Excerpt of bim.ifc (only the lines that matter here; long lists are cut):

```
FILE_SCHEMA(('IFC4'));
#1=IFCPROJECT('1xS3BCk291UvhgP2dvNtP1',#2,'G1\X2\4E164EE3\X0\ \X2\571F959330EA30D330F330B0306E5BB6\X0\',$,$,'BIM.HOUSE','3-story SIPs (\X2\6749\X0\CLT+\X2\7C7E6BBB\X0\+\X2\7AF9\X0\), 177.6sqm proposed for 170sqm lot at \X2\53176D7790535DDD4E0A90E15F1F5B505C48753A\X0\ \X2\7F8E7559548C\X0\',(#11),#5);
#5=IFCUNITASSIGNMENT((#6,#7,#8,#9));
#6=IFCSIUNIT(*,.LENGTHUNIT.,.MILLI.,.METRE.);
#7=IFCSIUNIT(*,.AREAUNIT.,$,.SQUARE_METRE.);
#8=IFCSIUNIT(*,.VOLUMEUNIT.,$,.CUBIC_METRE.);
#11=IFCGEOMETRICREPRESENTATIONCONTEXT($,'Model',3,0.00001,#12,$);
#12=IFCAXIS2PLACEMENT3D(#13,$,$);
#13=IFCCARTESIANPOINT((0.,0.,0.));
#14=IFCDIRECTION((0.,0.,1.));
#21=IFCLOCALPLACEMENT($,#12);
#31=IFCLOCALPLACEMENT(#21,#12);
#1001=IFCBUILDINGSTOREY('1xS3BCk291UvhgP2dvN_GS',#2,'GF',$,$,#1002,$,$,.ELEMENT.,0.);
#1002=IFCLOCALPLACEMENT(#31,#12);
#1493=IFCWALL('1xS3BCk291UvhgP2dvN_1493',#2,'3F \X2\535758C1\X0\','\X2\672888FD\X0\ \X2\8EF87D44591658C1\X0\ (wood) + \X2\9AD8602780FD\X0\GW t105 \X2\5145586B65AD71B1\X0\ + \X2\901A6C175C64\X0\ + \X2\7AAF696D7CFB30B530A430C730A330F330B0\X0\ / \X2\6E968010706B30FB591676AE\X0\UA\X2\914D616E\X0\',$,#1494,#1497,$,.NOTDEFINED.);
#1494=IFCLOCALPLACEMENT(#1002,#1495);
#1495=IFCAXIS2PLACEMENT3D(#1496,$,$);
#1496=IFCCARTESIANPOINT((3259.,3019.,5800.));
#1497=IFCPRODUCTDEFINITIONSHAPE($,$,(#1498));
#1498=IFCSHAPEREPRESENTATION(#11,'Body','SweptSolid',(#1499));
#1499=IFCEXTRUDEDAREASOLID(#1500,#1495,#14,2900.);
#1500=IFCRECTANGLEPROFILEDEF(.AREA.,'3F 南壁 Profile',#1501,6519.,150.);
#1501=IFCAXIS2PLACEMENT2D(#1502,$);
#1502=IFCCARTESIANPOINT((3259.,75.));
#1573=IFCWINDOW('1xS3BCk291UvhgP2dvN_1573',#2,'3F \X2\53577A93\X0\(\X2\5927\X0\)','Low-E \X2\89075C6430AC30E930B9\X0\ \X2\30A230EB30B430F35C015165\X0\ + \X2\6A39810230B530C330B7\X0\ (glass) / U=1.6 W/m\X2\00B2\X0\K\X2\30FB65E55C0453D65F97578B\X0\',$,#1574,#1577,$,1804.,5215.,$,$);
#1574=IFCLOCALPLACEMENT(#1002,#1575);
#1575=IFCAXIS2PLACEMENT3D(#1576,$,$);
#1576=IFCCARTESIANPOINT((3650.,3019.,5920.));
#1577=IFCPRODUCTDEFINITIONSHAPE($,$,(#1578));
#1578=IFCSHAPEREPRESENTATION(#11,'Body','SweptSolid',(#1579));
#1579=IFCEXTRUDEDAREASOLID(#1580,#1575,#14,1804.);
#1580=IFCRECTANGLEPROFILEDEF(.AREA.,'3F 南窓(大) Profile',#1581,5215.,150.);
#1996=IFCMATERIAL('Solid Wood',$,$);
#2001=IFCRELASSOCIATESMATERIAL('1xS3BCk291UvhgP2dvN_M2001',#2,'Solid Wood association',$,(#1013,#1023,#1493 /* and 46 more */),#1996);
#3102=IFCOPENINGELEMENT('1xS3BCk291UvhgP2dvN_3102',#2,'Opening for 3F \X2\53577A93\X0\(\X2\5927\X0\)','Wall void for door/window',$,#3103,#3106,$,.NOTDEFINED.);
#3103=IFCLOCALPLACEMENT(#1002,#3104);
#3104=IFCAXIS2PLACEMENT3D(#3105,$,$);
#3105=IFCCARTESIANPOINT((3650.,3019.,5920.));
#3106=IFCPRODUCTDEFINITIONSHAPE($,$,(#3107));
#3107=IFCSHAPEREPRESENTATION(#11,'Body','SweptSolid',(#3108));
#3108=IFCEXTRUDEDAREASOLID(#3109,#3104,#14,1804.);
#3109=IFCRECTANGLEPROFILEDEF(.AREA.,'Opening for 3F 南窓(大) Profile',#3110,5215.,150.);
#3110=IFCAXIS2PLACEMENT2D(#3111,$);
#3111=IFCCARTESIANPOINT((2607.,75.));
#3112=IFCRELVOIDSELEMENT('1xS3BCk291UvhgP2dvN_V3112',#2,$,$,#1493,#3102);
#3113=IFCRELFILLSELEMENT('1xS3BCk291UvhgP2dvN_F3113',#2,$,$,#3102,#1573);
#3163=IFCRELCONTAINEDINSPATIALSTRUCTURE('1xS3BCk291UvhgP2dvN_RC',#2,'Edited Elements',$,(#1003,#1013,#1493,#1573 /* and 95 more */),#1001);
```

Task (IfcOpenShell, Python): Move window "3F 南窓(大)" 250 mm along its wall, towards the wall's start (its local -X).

```python
import ifcopenshell
import ifcopenshell.api.geometry
import ifcopenshell.util.placement
import ifcopenshell.util.unit

model = ifcopenshell.open("bim.ifc")
unit_scale = ifcopenshell.util.unit.calculate_unit_scale(model)

window = model.by_guid("1xS3BCk291UvhgP2dvN_1573")
opening = window.FillsVoids[0].RelatingOpeningElement
wall = opening.VoidsElements[0].RelatingBuildingElement

wall_matrix = ifcopenshell.util.placement.get_local_placement(wall.ObjectPlacement)
shift = wall_matrix[:3, 0] * -0.25 / unit_scale
before = ifcopenshell.util.placement.get_local_placement(window.ObjectPlacement)[:3, 3].copy()

# The window is not placed relative to its opening, so move both.
for product in (opening, window):
    matrix = ifcopenshell.util.placement.get_local_placement(product.ObjectPlacement)
    matrix[:3, 3] += shift
    ifcopenshell.api.geometry.edit_object_placement(model, product=product, matrix=matrix, is_si=False)

after = ifcopenshell.util.placement.get_local_placement(window.ObjectPlacement)[:3, 3]
print("window moved by", (after - before).round(3) + 0.0)

model.write("bim_updated.ifc")
```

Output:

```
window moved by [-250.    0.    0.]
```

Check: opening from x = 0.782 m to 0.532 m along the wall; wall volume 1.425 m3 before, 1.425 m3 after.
